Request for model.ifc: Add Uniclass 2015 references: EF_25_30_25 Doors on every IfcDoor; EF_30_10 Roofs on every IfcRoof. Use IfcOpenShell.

First a look at what the model holds.

```python
import ifcopenshell

model = ifcopenshell.open("model.ifc")
print(model.schema)
print("classifications:", [c.Name for c in model.by_type("IfcClassification")])
for ifc_class in ("IfcDoor", "IfcRoof", "IfcStair", "IfcWall", "IfcWindow"):
    print(ifc_class, len(model.by_type(ifc_class)))
```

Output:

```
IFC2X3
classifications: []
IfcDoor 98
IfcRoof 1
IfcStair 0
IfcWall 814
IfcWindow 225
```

```python
import ifcopenshell
import ifcopenshell.api.classification

model = ifcopenshell.open("model.ifc")

# IFC2X3 requires Source and Edition and has no link from the project to the system.
system = model.create_entity("IfcClassification", Source="NBS", Edition="2015", Name="Uniclass 2015")

codes = {
    "IfcDoor": ("EF_25_30_25", "Doors"),
    "IfcRoof": ("EF_30_10", "Roofs"),
}
for ifc_class, (code, name) in codes.items():
    products = model.by_type(ifc_class)
    ifcopenshell.api.classification.add_reference(
        model, products=products, classification=system, identification=code, name=name
    )
    print(code, len(products))

model.write("model_edited.ifc")
```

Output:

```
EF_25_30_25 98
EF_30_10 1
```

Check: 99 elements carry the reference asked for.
